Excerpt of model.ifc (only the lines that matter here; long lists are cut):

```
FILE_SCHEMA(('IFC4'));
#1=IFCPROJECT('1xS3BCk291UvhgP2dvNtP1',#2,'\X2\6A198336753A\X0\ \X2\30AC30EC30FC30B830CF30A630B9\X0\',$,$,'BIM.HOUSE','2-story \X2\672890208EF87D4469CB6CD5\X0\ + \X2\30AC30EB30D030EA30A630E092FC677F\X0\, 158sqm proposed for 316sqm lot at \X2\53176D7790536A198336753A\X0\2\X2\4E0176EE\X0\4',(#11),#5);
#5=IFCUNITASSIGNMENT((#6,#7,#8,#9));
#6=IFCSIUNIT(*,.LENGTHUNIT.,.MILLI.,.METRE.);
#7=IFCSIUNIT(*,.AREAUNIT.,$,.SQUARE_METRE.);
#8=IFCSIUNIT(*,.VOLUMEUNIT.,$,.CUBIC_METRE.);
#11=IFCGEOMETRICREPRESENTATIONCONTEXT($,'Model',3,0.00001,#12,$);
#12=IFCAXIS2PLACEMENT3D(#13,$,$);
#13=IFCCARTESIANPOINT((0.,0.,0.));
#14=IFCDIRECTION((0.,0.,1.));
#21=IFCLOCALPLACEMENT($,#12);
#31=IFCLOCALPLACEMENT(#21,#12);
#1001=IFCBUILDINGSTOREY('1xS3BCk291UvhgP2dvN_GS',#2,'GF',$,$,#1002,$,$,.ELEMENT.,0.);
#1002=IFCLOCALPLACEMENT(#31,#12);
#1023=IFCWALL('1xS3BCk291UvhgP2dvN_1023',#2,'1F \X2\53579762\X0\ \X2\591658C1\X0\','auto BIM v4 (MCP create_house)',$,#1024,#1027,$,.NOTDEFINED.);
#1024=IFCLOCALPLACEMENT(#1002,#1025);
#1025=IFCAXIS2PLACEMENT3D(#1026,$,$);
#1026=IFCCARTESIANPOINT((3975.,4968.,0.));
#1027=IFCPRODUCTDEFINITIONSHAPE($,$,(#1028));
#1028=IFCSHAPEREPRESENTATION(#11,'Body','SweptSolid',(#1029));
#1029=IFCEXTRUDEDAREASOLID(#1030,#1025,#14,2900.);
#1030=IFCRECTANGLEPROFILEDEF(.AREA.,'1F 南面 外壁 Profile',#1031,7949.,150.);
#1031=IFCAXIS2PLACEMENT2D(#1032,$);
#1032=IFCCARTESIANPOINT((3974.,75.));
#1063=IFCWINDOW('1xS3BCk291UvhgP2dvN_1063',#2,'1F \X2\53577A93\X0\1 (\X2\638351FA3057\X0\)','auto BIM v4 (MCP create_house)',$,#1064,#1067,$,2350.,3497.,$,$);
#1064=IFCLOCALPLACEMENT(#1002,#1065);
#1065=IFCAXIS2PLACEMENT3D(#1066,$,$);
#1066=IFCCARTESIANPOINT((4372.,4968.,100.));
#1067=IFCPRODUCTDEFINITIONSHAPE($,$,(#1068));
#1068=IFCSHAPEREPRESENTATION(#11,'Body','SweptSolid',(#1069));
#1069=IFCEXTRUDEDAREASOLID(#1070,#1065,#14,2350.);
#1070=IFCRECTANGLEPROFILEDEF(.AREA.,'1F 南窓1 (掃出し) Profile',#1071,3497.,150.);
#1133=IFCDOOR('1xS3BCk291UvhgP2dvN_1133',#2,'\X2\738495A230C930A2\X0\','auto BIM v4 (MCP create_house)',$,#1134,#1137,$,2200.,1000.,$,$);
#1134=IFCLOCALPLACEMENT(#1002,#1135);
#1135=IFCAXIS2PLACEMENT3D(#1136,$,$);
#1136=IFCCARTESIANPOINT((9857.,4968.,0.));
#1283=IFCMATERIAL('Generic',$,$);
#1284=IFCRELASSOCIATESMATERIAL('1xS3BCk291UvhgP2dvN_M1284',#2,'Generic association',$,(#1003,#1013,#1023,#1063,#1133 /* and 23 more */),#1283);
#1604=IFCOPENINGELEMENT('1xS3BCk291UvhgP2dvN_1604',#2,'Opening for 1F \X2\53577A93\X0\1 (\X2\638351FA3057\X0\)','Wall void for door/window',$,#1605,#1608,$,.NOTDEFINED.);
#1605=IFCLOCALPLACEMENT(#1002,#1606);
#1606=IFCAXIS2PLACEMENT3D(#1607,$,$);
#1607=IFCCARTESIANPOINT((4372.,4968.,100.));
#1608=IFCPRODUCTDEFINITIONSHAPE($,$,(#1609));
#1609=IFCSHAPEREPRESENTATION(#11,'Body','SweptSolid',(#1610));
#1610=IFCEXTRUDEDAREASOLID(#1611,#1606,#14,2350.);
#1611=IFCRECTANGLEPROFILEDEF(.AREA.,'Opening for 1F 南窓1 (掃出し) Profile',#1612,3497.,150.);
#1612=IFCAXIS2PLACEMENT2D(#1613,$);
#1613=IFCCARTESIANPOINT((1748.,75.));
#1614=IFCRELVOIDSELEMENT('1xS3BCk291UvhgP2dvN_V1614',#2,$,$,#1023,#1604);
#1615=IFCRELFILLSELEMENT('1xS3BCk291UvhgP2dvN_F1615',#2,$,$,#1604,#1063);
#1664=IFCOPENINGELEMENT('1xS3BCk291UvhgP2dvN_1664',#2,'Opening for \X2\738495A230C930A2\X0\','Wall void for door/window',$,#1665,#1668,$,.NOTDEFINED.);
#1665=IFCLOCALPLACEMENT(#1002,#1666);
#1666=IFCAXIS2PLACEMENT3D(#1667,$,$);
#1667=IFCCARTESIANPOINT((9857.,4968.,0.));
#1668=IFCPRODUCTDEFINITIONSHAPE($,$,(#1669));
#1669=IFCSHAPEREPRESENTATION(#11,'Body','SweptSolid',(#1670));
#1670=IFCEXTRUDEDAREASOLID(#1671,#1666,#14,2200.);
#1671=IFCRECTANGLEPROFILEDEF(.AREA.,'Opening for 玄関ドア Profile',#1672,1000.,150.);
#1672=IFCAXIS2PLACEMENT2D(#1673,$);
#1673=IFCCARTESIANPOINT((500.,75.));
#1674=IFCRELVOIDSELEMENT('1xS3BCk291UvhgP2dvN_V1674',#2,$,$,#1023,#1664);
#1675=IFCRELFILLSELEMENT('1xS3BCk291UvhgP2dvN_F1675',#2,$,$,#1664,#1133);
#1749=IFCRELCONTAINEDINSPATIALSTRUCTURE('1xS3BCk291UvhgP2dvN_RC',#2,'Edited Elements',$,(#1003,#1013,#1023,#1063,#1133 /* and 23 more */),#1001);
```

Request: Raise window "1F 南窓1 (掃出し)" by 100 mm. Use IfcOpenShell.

```python
import numpy as np
import ifcopenshell
import ifcopenshell.api.geometry
import ifcopenshell.util.placement
import ifcopenshell.util.unit

model = ifcopenshell.open("model.ifc")
unit_scale = ifcopenshell.util.unit.calculate_unit_scale(model)

window = model.by_id(1063)
opening = window.FillsVoids[0].RelatingOpeningElement
dz = 0.1 / unit_scale

shift = np.array([0.0, 0.0, dz])
# The window is not placed relative to its opening, so move both.
for product in (opening, window):
    matrix = ifcopenshell.util.placement.get_local_placement(product.ObjectPlacement)
    matrix[:3, 3] += shift
    ifcopenshell.api.geometry.edit_object_placement(model, product=product, matrix=matrix, is_si=False)

print(f"moved by {dz * unit_scale:+.3f} m")

model.write("model-out.ifc")
```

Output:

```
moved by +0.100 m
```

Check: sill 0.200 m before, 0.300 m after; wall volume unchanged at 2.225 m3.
